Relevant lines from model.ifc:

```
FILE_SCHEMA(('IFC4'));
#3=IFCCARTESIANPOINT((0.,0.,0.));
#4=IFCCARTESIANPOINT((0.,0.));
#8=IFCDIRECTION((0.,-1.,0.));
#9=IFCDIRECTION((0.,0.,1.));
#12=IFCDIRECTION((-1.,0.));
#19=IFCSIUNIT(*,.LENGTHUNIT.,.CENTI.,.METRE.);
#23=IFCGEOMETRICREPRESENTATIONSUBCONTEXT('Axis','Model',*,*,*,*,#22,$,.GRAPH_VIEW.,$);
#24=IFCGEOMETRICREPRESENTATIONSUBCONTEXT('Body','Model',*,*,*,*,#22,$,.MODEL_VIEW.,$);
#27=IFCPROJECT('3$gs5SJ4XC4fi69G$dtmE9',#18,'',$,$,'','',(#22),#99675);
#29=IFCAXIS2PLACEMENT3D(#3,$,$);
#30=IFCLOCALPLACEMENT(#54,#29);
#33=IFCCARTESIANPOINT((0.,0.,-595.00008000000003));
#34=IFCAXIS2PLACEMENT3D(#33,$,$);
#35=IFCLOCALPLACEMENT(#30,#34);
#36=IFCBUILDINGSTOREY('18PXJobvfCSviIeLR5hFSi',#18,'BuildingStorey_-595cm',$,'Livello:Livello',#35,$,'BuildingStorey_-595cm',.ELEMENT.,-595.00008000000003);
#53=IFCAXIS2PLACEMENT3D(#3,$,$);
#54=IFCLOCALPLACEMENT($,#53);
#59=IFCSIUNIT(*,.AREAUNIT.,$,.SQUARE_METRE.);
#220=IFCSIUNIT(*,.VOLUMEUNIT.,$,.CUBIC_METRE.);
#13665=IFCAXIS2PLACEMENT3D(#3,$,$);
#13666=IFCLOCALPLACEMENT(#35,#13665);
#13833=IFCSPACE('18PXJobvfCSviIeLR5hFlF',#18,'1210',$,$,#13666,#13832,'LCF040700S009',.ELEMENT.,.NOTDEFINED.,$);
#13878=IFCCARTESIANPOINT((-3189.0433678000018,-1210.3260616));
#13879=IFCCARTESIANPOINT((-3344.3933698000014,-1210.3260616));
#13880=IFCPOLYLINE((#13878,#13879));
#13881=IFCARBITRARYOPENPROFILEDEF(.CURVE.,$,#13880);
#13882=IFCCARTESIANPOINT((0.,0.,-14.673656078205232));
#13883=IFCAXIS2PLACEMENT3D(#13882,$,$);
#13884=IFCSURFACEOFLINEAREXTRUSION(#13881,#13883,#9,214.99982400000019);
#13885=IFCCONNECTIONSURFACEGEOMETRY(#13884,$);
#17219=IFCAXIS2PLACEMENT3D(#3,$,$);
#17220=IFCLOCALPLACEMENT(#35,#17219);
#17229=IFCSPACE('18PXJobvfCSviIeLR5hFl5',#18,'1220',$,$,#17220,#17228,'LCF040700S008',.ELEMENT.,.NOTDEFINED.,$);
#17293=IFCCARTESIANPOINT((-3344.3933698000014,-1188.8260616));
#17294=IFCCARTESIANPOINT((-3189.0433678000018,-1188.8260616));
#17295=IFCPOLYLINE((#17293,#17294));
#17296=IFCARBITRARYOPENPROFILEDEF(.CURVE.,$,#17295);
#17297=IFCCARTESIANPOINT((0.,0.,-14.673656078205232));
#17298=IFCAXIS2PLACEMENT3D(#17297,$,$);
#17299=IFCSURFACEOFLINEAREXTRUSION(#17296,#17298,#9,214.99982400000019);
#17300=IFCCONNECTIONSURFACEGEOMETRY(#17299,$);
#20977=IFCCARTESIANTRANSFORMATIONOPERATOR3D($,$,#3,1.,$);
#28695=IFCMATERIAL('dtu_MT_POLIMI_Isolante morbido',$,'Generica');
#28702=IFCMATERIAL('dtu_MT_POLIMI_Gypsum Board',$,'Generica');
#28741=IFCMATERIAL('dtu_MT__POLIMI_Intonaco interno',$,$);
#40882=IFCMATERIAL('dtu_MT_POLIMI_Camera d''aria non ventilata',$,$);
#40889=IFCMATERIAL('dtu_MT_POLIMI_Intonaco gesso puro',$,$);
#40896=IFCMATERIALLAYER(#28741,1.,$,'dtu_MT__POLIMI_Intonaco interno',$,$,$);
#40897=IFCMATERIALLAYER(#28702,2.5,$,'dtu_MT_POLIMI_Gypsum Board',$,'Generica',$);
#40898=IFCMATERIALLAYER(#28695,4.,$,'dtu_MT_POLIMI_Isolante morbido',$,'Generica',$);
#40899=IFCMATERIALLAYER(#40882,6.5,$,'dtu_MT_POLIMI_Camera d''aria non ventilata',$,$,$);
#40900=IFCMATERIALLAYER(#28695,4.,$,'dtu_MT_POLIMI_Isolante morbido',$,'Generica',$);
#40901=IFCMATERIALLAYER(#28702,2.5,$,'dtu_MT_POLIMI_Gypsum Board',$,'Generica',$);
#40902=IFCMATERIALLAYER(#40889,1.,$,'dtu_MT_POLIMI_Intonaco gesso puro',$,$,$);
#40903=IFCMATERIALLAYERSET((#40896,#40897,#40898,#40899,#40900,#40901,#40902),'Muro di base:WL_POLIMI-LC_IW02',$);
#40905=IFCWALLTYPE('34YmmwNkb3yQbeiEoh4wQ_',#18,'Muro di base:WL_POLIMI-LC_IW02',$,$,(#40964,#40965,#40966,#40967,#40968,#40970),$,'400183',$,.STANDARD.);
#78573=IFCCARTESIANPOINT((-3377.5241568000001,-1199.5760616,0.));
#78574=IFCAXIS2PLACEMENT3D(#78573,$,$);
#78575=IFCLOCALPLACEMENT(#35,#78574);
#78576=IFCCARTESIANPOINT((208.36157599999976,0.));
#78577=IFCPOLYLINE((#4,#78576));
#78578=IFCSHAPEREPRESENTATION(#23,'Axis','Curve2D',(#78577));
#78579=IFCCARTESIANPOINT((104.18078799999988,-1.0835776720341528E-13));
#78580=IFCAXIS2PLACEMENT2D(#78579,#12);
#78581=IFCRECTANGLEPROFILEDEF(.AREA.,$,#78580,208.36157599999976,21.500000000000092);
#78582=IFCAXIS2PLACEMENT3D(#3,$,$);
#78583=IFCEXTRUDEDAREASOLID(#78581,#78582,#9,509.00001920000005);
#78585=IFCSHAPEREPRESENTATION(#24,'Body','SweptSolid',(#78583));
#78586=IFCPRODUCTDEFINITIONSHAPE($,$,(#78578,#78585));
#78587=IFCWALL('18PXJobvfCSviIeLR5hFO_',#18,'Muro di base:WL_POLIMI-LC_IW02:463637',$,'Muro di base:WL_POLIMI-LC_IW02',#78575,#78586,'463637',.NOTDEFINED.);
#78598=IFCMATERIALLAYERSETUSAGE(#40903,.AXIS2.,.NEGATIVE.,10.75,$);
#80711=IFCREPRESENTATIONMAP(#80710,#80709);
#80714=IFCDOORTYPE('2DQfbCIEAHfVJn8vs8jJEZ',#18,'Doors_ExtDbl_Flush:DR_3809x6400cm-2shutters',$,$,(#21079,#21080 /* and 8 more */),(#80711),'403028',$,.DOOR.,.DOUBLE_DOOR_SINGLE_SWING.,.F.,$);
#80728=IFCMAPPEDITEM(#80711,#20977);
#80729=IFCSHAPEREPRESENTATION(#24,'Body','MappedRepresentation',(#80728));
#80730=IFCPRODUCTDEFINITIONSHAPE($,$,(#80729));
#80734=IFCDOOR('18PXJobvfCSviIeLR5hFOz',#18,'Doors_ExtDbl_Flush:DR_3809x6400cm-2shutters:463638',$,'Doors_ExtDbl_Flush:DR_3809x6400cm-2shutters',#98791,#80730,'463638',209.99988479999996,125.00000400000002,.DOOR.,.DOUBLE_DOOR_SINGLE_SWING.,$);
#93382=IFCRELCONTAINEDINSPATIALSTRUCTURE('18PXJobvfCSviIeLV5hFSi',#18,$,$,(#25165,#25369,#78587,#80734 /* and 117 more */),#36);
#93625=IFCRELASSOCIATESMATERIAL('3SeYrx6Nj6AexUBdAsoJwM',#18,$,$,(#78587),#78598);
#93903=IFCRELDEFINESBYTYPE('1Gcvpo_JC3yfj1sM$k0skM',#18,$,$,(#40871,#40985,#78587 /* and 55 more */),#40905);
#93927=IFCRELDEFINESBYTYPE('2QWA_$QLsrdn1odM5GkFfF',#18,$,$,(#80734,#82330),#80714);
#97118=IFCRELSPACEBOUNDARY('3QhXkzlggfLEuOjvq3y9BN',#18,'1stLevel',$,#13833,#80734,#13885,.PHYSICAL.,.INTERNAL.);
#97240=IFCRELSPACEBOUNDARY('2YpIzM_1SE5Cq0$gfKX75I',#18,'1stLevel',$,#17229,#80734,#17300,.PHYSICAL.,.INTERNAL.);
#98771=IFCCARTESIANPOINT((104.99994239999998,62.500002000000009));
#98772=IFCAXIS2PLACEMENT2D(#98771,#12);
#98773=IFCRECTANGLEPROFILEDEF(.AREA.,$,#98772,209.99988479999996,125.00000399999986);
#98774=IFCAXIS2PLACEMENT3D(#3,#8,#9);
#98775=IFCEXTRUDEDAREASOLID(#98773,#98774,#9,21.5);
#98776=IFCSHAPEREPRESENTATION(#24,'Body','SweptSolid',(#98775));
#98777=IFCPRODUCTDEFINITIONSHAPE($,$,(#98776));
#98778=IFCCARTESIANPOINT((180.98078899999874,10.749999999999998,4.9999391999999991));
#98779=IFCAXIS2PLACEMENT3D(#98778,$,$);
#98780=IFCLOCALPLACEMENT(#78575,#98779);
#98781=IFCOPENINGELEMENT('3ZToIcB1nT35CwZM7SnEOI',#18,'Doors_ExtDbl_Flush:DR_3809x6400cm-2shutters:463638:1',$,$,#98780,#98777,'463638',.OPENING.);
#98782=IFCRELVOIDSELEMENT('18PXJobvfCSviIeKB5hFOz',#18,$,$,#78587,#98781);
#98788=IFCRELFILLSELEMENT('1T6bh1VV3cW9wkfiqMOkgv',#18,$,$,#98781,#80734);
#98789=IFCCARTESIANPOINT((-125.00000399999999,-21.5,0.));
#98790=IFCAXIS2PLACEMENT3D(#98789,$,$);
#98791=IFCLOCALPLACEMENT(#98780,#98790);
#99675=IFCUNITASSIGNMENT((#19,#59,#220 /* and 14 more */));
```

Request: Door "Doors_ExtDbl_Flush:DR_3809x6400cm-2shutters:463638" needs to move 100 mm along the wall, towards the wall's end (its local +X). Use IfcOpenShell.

```python
import numpy as np
import ifcopenshell
import ifcopenshell.api.geometry
import ifcopenshell.util.placement
import ifcopenshell.util.unit

model = ifcopenshell.open("model.ifc")
unit_scale = ifcopenshell.util.unit.calculate_unit_scale(model)

door = model.by_id(80734)
opening = door.FillsVoids[0].RelatingOpeningElement
wall = opening.VoidsElements[0].RelatingBuildingElement

wall_matrix = ifcopenshell.util.placement.get_local_placement(wall.ObjectPlacement)
shift = wall_matrix[:3, 0] * 0.1 / unit_scale
before = ifcopenshell.util.placement.get_local_placement(door.ObjectPlacement)[:3, 3].copy()

# The door is placed relative to its opening, so it follows when the opening moves.
matrix = ifcopenshell.util.placement.get_local_placement(opening.ObjectPlacement)
matrix[:3, 3] += shift
ifcopenshell.api.geometry.edit_object_placement(
    model, product=opening, matrix=matrix, is_si=False, should_transform_children=True
)

# Space boundary surfaces are stored in each space's coordinates; move them too.
for rel in door.ProvidesBoundaries:
    if not rel.ConnectionGeometry:
        continue
    surface = rel.ConnectionGeometry.SurfaceOnRelatingElement
    space_matrix = ifcopenshell.util.placement.get_local_placement(rel.RelatingSpace.ObjectPlacement)
    point = np.array(surface.Position.Location.Coordinates) + space_matrix[:3, :3].T @ shift
    surface.Position = model.createIfcAxis2Placement3D(
        model.createIfcCartesianPoint(point.tolist()), surface.Position.Axis, surface.Position.RefDirection
    )

after = ifcopenshell.util.placement.get_local_placement(door.ObjectPlacement)[:3, 3]
print("door moved by", (after - before).round(3) + 0.0)

model.write("model-out.ifc")
```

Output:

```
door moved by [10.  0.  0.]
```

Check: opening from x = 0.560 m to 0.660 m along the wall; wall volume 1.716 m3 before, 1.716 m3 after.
